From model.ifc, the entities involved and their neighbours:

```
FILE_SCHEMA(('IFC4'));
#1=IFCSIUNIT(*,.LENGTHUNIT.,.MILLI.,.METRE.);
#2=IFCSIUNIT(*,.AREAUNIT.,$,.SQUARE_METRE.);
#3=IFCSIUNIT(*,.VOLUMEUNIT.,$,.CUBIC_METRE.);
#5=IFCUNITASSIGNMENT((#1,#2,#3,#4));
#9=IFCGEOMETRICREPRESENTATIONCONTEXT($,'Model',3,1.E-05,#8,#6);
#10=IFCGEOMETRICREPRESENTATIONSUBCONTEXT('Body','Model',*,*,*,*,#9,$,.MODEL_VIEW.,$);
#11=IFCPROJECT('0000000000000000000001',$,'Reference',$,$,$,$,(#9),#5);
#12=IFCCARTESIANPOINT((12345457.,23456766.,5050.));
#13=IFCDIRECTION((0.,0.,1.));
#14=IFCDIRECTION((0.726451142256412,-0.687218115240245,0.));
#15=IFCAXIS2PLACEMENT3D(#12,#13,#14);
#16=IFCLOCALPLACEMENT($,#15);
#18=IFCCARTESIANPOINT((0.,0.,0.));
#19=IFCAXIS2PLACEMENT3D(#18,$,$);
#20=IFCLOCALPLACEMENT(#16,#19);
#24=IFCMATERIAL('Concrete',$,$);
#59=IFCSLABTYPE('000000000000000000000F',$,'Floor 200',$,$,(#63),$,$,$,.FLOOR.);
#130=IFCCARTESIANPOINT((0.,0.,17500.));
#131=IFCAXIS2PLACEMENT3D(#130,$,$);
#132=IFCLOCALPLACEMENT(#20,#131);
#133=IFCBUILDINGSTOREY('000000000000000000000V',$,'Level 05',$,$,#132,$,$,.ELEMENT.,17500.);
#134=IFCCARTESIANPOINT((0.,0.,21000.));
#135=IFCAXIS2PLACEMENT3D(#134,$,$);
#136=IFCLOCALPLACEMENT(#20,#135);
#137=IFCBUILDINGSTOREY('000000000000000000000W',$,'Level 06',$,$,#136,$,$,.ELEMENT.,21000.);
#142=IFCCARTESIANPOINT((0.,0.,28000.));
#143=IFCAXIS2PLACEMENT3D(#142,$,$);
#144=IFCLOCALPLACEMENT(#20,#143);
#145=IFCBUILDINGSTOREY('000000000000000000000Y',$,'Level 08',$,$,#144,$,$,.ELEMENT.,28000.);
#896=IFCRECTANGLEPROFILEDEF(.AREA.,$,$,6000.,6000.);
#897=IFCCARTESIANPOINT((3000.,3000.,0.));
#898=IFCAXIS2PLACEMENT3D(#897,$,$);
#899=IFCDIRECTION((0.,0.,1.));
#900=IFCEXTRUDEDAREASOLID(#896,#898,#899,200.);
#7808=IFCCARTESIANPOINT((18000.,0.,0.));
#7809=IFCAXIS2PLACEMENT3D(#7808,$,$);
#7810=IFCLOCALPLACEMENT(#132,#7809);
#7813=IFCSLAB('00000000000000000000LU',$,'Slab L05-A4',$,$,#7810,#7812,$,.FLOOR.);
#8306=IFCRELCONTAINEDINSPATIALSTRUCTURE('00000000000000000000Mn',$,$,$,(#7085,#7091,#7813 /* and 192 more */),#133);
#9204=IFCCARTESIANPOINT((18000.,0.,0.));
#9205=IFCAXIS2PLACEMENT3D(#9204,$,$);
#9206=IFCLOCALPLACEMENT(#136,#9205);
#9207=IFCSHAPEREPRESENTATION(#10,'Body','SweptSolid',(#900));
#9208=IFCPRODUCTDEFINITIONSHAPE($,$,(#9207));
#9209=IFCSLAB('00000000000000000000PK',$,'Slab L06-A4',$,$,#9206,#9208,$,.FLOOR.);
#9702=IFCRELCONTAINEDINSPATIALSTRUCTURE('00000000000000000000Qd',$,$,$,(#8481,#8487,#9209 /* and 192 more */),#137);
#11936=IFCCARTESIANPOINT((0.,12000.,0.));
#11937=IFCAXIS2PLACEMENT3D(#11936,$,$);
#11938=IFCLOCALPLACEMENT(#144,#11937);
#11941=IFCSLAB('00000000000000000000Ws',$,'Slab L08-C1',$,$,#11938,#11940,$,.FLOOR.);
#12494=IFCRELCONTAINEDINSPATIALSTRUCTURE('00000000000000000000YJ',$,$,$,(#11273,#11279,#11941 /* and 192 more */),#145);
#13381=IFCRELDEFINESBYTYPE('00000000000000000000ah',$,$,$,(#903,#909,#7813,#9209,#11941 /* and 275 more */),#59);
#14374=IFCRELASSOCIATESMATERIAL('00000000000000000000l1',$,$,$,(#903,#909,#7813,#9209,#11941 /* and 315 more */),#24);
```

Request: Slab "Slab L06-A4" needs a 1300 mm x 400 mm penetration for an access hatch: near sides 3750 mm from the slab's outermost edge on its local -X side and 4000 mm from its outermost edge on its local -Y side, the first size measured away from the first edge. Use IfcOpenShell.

```python
import numpy as np
import ifcopenshell
import ifcopenshell.api.feature
import ifcopenshell.api.geometry
import ifcopenshell.api.root
import ifcopenshell.geom
import ifcopenshell.util.placement
import ifcopenshell.util.representation
import ifcopenshell.util.shape
import ifcopenshell.util.unit

model = ifcopenshell.open("model.ifc")
unit_scale = ifcopenshell.util.unit.calculate_unit_scale(model)
settings = ifcopenshell.geom.settings()


def volume(element):
    """Net volume in cubic metres, openings subtracted."""
    shape = ifcopenshell.geom.create_shape(settings, element)
    return ifcopenshell.util.shape.get_volume(shape.geometry)


slab = model.by_guid("00000000000000000000PK")
before = volume(slab)

# Extent in the slab's own axes, in metres. The edges named are its -X and -Y sides.
slab_shape = ifcopenshell.geom.create_shape(settings, slab)
vertices = ifcopenshell.util.shape.get_vertices(slab_shape.geometry)
x_min, y_min, bottom = vertices.min(axis=0)
top = vertices[:, 2].max()

opening = ifcopenshell.api.root.create_entity(model, ifc_class="IfcOpeningElement", name="Access hatch opening", predefined_type="OPENING")
context = ifcopenshell.util.representation.get_context(model, "Model", "Body", "MODEL_VIEW")
width, depth = 1.3, 0.4
outline = [(0.0, 0.0), (width, 0.0), (width, depth), (0.0, depth), (0.0, 0.0)]
# Overshoot both faces by 50 mm so the cut is clean.
shape = ifcopenshell.api.geometry.add_slab_representation(
    model, context=context, depth=top - bottom + 0.1, polyline=outline
)
ifcopenshell.api.geometry.assign_representation(model, product=opening, representation=shape)

matrix = ifcopenshell.util.placement.get_local_placement(slab.ObjectPlacement)
matrix[:, 3] = matrix @ np.append(np.array([x_min + 3.75, y_min + 4, bottom - 0.05]) / unit_scale, 1.0)
ifcopenshell.api.geometry.edit_object_placement(model, product=opening, matrix=matrix, is_si=False)
ifcopenshell.api.feature.add_feature(model, feature=opening, element=slab)

after = volume(slab)

print(f"slab volume {before:.3f} -> {after:.3f} m3")

model.write("model_edited.ifc")
```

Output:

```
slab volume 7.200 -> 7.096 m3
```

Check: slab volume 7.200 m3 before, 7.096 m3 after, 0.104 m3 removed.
